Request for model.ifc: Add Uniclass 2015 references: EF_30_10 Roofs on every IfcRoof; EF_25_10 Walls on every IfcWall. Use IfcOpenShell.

First a look at what the model holds.

```python
import ifcopenshell

model = ifcopenshell.open("model.ifc")
print(model.schema)
print("classifications:", [c.Name for c in model.by_type("IfcClassification")])
for ifc_class in ("IfcDoor", "IfcRoof", "IfcStair", "IfcWall", "IfcWindow"):
    print(ifc_class, len(model.by_type(ifc_class)))
```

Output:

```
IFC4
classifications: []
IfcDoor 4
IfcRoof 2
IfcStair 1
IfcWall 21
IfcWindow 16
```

```python
import ifcopenshell
import ifcopenshell.api.classification

model = ifcopenshell.open("model.ifc")

system = ifcopenshell.api.classification.add_classification(model, classification="Uniclass 2015")

codes = {
    "IfcRoof": ("EF_30_10", "Roofs"),
    "IfcWall": ("EF_25_10", "Walls"),
}
for ifc_class, (code, name) in codes.items():
    products = model.by_type(ifc_class)
    ifcopenshell.api.classification.add_reference(
        model, products=products, classification=system, identification=code, name=name
    )
    print(code, len(products))

model.write("model_v2.ifc")
```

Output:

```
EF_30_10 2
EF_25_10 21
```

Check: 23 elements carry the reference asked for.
